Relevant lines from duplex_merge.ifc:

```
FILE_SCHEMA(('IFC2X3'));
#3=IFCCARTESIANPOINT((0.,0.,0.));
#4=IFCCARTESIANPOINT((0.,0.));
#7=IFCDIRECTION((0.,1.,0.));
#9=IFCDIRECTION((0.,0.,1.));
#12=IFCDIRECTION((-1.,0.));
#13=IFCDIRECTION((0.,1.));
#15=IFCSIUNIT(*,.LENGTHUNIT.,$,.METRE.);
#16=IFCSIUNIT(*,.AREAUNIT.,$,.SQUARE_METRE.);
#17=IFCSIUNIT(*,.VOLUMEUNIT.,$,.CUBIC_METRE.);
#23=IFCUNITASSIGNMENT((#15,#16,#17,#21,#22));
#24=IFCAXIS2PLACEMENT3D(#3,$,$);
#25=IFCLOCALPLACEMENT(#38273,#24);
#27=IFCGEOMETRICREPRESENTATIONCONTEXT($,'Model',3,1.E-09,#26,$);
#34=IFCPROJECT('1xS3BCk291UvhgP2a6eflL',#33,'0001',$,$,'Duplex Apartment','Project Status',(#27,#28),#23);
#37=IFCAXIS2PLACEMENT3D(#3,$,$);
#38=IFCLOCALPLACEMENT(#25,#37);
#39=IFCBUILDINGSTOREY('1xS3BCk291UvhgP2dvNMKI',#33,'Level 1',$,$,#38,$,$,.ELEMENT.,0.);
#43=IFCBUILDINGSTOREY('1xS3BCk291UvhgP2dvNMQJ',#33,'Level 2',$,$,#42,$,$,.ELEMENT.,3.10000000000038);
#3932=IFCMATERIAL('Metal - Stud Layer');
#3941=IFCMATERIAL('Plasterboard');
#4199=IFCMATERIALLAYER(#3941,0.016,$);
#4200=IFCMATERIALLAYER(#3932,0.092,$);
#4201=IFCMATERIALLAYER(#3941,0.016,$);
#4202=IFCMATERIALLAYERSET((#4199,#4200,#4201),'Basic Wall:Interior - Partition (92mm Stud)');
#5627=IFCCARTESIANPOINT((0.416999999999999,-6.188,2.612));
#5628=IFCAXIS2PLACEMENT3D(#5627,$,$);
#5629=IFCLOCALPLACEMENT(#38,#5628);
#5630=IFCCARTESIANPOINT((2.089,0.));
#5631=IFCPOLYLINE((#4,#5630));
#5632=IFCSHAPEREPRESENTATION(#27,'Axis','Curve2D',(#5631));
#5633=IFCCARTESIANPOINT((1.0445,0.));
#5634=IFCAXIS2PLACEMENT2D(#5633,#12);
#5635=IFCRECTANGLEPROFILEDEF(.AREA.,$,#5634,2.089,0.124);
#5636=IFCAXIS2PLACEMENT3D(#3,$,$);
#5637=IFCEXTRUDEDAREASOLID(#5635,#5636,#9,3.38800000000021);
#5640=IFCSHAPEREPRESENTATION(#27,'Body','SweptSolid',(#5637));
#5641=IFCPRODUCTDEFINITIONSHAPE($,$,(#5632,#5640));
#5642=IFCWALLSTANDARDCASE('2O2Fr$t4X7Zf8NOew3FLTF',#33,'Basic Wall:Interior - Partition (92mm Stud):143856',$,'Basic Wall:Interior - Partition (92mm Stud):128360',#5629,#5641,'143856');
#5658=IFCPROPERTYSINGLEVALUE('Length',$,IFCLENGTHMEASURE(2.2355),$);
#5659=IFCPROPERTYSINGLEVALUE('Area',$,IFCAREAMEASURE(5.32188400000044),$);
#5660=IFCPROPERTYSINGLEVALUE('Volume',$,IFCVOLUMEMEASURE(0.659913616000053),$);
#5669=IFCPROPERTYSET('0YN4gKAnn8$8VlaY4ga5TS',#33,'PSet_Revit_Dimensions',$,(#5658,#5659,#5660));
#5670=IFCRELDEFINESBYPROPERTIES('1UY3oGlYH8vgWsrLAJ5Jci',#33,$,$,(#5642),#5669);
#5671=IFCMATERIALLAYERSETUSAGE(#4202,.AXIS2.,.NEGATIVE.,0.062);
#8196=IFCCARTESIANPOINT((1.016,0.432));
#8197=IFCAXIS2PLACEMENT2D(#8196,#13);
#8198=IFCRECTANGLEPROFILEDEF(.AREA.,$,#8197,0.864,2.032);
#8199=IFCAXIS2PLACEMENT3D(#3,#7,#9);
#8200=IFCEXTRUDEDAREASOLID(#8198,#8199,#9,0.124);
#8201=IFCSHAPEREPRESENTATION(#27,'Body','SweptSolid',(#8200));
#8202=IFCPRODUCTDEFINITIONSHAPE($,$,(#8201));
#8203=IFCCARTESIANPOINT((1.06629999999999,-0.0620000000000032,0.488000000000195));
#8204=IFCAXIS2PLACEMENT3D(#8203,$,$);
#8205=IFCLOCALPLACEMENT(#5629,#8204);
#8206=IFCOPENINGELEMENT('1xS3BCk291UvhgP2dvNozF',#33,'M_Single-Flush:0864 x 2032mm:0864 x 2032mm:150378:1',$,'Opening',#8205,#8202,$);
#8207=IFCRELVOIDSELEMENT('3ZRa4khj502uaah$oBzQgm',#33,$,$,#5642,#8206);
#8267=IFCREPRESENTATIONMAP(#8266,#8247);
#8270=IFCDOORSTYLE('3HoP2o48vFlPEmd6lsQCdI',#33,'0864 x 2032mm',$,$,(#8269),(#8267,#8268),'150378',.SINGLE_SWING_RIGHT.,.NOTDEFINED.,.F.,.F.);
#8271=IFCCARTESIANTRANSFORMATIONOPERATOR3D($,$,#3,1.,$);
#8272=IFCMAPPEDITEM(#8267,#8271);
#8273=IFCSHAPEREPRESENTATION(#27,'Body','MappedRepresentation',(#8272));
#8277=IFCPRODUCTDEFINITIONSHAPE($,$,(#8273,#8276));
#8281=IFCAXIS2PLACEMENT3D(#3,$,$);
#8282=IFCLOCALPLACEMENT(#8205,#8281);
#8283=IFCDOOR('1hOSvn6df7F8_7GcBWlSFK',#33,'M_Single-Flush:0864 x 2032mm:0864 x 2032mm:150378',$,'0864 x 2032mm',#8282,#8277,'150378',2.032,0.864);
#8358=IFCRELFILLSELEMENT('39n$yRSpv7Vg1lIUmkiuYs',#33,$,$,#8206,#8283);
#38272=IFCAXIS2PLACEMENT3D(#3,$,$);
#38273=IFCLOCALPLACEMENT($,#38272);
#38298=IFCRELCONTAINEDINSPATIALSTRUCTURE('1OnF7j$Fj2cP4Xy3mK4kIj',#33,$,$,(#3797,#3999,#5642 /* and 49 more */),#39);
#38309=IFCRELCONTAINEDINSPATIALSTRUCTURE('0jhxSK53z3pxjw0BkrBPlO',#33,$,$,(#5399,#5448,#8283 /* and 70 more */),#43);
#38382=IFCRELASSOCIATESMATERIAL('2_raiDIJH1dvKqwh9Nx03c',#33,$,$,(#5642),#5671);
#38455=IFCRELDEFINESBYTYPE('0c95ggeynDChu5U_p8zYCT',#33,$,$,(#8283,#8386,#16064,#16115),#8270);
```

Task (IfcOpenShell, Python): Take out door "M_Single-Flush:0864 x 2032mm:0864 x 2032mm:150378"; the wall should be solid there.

```python
import ifcopenshell
import ifcopenshell.api.feature
import ifcopenshell.api.pset
import ifcopenshell.api.root
import ifcopenshell.geom
import ifcopenshell.util.element
import ifcopenshell.util.shape
import ifcopenshell.util.unit

model = ifcopenshell.open("duplex_merge.ifc")
area_scale = ifcopenshell.util.unit.calculate_unit_scale(model, "AREAUNIT")
volume_scale = ifcopenshell.util.unit.calculate_unit_scale(model, "VOLUMEUNIT")
settings = ifcopenshell.geom.settings()


def volume(element):
    """Net volume in cubic metres, openings subtracted."""
    shape = ifcopenshell.geom.create_shape(settings, element)
    return ifcopenshell.util.shape.get_volume(shape.geometry)


door = model.by_guid("1hOSvn6df7F8_7GcBWlSFK")
opening = door.FillsVoids[0].RelatingOpeningElement
wall = opening.VoidsElements[0].RelatingBuildingElement
before = volume(wall)

ifcopenshell.api.root.remove_product(model, product=door)
ifcopenshell.api.feature.remove_feature(model, feature=opening)

after = volume(wall)
thickness = 0.124  # wall thickness in metres

# Update the wall's stored quantities.
pset = model.by_id(ifcopenshell.util.element.get_pset(wall, "PSet_Revit_Dimensions", should_inherit=False)["id"])
ifcopenshell.api.pset.edit_pset(model, pset=pset, properties={
    "Area": model.create_entity("IfcAreaMeasure", after / thickness / area_scale),
    "Volume": model.create_entity("IfcVolumeMeasure", after / volume_scale),
})

print(f"wall volume {before:.3f} -> {after:.3f} m3")

model.write("duplex_merge-out.ifc")
```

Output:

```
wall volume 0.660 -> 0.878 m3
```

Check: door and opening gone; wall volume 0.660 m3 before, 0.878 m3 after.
